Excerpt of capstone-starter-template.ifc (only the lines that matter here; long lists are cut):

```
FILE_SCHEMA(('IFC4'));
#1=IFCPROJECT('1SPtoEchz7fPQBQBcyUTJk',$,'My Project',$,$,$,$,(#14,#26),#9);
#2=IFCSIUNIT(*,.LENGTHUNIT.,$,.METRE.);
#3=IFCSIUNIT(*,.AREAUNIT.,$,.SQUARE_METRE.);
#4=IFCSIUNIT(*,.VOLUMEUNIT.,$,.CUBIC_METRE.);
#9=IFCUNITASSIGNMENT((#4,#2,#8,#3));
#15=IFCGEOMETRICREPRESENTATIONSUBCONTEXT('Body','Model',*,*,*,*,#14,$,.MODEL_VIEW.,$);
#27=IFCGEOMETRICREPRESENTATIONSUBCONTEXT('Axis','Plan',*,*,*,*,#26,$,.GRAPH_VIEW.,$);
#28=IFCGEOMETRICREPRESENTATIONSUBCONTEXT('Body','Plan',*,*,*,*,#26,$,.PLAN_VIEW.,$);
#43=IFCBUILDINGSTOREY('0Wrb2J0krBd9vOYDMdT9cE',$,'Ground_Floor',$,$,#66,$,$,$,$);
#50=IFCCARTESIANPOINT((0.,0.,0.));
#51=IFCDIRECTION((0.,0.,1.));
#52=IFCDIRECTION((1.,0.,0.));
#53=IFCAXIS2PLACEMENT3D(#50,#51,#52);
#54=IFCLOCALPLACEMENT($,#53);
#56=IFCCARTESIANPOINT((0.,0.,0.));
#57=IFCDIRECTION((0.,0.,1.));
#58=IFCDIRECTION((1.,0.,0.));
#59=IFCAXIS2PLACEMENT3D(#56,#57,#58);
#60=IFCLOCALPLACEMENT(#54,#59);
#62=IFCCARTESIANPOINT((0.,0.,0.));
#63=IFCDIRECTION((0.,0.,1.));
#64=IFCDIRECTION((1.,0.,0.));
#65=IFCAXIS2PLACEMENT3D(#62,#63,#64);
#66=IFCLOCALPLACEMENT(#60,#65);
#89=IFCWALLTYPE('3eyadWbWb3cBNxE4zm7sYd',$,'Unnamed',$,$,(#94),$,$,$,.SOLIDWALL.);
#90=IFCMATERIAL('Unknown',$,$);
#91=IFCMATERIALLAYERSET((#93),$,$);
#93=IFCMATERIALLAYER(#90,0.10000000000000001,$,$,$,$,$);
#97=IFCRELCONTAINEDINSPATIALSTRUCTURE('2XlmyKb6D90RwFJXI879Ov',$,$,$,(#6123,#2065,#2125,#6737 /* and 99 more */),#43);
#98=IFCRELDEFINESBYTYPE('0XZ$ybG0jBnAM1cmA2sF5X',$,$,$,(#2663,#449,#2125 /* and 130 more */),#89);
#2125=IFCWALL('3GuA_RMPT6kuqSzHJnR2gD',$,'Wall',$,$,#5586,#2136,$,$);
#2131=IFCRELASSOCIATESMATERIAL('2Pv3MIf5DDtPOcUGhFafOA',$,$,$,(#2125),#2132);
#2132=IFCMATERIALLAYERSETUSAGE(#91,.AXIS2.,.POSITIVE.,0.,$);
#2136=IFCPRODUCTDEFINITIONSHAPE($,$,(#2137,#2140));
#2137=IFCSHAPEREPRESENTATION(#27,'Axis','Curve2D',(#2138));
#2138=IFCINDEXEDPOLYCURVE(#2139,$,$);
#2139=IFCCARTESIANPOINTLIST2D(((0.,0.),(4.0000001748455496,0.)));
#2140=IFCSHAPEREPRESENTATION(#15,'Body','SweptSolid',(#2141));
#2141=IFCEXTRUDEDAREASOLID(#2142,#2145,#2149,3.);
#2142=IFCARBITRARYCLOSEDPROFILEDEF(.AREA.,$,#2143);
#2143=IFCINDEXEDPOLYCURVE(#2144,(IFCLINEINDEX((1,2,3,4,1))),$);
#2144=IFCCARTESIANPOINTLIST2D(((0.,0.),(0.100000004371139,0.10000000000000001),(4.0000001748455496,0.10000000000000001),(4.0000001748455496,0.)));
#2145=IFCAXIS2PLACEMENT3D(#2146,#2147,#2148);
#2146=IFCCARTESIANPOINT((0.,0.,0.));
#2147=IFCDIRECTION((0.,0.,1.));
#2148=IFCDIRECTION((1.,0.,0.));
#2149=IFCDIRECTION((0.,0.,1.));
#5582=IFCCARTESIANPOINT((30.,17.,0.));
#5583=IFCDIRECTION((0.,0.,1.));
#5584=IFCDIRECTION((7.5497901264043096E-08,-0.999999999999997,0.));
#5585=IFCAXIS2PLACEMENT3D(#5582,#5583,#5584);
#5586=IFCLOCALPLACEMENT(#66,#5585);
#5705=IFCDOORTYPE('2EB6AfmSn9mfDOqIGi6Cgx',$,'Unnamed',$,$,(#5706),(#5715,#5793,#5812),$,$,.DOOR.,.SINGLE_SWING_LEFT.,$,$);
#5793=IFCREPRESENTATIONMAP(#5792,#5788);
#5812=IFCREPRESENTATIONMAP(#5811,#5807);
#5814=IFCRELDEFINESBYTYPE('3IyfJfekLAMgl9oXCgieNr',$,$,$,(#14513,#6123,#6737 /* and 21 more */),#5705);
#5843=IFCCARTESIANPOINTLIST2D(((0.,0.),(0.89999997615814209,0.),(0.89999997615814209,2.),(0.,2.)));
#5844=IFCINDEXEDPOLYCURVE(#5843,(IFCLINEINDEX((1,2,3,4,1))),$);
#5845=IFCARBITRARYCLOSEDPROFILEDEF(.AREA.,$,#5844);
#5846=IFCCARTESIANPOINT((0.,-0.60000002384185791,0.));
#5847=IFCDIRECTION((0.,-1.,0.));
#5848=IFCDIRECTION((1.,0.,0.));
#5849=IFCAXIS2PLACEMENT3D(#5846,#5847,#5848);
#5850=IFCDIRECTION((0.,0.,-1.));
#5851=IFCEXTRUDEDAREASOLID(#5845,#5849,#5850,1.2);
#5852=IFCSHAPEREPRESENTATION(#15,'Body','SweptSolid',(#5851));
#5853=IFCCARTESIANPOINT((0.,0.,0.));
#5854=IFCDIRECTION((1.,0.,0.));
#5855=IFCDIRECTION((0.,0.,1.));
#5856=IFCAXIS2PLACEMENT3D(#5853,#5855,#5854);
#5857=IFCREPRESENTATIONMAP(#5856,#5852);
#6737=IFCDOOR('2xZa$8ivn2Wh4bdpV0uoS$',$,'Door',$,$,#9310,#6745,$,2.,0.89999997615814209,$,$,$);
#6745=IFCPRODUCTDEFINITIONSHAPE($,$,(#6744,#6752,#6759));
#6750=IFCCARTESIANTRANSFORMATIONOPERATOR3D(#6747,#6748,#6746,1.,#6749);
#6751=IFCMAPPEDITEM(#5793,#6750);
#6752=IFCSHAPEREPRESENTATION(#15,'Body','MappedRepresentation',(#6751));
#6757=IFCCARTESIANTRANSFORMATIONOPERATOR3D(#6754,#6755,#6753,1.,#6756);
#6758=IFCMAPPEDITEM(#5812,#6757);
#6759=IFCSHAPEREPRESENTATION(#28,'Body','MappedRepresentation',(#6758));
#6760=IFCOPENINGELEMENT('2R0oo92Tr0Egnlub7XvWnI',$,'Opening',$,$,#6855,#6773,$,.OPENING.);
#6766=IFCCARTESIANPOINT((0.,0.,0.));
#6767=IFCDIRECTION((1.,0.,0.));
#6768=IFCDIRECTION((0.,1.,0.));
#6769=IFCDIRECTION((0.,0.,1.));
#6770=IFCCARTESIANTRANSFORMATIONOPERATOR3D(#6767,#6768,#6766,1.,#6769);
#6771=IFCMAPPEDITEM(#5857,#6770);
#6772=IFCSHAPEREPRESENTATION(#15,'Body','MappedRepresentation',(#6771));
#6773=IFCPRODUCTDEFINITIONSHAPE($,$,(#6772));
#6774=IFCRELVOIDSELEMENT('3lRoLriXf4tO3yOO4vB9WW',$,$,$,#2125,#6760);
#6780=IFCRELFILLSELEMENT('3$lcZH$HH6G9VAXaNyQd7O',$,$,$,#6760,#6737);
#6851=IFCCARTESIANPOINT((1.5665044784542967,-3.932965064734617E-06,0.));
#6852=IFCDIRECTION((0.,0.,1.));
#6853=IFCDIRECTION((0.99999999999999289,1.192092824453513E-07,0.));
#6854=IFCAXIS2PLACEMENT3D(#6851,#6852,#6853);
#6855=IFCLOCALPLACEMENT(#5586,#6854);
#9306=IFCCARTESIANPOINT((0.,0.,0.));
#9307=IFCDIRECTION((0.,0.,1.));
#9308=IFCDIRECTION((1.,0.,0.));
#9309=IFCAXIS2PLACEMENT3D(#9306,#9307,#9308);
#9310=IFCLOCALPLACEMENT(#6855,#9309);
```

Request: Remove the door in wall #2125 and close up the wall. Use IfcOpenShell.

```python
import ifcopenshell
import ifcopenshell.api.feature
import ifcopenshell.api.root
import ifcopenshell.geom
import ifcopenshell.util.shape

model = ifcopenshell.open("capstone-starter-template.ifc")
settings = ifcopenshell.geom.settings()


def volume(element):
    """Net volume in cubic metres, openings subtracted."""
    shape = ifcopenshell.geom.create_shape(settings, element)
    return ifcopenshell.util.shape.get_volume(shape.geometry)


door = model.by_guid("2xZa$8ivn2Wh4bdpV0uoS$")
opening = door.FillsVoids[0].RelatingOpeningElement
wall = opening.VoidsElements[0].RelatingBuildingElement
before = volume(wall)

ifcopenshell.api.root.remove_product(model, product=door)
ifcopenshell.api.feature.remove_feature(model, feature=opening)

after = volume(wall)

print(f"wall volume {before:.3f} -> {after:.3f} m3")

model.write("capstone-starter-template-out.ifc")
```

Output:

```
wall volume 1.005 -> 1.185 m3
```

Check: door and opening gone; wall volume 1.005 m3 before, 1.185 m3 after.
